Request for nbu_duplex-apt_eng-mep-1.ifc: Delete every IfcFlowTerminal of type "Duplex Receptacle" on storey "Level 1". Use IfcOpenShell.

First a look at what the model holds.

```python
import ifcopenshell
import ifcopenshell.util.element

model = ifcopenshell.open("nbu_duplex-apt_eng-mep-1.ifc")
print(model.schema)
storey = next(s for s in model.by_type("IfcBuildingStorey") if s.Name == "Level 1")
terminals = [e for e in ifcopenshell.util.element.get_decomposition(storey) if e.is_a("IfcFlowTerminal")]
seen = {}
for e in terminals:
    element_type = ifcopenshell.util.element.get_type(e)
    name = element_type.Name if element_type not in (None, e) else None
    seen[name] = seen.get(name, 0) + 1
for name, count in sorted(seen.items(), key=str):
    print(count, "x", name)
```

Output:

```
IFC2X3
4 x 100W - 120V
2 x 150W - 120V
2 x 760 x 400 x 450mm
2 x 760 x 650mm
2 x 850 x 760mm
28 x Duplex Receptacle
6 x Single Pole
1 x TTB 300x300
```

```python
import ifcopenshell
import ifcopenshell.api.root
import ifcopenshell.util.element

model = ifcopenshell.open("nbu_duplex-apt_eng-mep-1.ifc")

storey = next(s for s in model.by_type("IfcBuildingStorey") if s.Name == "Level 1")
terminals = [e for e in ifcopenshell.util.element.get_decomposition(storey) if e.is_a("IfcFlowTerminal")]
targets = [e for e in terminals if (t := ifcopenshell.util.element.get_type(e)) not in (None, e) and t.Name == "Duplex Receptacle"]

for e in targets:
    ifcopenshell.api.root.remove_product(model, product=e)
print(len(targets), "removed")

model.write("nbu_duplex-apt_eng-mep-1-out.ifc")
```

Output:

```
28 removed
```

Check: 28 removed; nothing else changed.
